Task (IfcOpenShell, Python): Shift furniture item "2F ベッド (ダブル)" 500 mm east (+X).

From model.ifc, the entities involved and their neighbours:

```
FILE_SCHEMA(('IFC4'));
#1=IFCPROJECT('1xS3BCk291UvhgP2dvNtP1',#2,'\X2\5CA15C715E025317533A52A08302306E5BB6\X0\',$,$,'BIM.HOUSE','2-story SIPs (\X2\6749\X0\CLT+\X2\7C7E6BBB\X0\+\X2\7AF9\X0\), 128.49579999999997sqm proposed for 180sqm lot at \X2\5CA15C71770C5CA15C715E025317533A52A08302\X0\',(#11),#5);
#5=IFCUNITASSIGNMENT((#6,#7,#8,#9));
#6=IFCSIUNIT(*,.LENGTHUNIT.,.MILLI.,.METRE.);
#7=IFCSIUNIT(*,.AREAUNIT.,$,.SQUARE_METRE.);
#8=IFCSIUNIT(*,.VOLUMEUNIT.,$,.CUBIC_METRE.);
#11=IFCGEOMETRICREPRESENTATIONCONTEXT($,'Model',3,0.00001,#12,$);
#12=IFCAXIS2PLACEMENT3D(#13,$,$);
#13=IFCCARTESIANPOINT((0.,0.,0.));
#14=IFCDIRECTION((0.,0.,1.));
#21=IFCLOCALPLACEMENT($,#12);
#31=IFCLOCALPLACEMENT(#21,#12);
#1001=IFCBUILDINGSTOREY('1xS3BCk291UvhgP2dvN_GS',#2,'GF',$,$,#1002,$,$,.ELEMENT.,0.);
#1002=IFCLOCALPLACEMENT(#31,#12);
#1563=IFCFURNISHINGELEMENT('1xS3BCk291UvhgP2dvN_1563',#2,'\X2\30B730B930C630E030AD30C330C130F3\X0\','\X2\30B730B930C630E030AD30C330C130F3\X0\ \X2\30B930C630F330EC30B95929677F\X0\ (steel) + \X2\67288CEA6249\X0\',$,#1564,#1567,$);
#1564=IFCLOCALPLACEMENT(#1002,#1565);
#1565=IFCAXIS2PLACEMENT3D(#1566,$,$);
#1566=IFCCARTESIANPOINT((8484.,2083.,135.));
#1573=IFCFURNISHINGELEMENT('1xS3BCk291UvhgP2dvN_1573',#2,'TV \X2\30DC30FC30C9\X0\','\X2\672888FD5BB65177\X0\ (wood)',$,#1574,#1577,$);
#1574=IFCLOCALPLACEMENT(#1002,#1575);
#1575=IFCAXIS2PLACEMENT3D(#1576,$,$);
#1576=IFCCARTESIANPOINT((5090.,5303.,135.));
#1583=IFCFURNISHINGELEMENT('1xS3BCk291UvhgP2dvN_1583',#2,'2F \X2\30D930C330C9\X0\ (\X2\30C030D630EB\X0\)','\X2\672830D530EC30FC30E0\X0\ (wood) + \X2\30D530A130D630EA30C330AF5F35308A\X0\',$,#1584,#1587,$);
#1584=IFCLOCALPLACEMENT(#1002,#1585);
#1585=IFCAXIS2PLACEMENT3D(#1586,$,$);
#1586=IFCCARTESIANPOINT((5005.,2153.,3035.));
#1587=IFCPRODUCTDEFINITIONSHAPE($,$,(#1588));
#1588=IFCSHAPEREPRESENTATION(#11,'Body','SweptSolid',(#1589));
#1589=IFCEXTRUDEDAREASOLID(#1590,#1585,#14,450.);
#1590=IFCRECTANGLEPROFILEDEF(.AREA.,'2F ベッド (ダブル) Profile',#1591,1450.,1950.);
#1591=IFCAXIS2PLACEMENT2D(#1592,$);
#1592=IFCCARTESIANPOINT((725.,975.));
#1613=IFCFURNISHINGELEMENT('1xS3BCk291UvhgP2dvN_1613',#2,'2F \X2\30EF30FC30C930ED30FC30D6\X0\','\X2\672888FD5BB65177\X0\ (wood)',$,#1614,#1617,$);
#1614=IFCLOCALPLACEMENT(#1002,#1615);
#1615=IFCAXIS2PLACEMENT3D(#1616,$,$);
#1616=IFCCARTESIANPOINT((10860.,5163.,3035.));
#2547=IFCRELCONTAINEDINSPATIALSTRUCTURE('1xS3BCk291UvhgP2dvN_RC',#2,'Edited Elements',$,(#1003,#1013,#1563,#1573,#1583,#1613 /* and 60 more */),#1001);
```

```python
import ifcopenshell
import ifcopenshell.api.geometry
import ifcopenshell.util.placement
import ifcopenshell.util.unit

model = ifcopenshell.open("model.ifc")
unit_scale = ifcopenshell.util.unit.calculate_unit_scale(model)

item = model.by_guid("1xS3BCk291UvhgP2dvN_1583")
matrix = ifcopenshell.util.placement.get_local_placement(item.ObjectPlacement)
matrix[0, 3] += 0.5 / unit_scale
ifcopenshell.api.geometry.edit_object_placement(model, product=item, matrix=matrix, is_si=False)

print(ifcopenshell.util.placement.get_local_placement(item.ObjectPlacement).round(3) + 0.0)

model.write("model_edited.ifc")
```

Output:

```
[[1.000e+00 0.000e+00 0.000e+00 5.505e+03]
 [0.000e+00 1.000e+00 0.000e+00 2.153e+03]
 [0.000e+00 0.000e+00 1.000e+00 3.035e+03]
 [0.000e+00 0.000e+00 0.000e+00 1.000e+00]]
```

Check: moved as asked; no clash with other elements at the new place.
